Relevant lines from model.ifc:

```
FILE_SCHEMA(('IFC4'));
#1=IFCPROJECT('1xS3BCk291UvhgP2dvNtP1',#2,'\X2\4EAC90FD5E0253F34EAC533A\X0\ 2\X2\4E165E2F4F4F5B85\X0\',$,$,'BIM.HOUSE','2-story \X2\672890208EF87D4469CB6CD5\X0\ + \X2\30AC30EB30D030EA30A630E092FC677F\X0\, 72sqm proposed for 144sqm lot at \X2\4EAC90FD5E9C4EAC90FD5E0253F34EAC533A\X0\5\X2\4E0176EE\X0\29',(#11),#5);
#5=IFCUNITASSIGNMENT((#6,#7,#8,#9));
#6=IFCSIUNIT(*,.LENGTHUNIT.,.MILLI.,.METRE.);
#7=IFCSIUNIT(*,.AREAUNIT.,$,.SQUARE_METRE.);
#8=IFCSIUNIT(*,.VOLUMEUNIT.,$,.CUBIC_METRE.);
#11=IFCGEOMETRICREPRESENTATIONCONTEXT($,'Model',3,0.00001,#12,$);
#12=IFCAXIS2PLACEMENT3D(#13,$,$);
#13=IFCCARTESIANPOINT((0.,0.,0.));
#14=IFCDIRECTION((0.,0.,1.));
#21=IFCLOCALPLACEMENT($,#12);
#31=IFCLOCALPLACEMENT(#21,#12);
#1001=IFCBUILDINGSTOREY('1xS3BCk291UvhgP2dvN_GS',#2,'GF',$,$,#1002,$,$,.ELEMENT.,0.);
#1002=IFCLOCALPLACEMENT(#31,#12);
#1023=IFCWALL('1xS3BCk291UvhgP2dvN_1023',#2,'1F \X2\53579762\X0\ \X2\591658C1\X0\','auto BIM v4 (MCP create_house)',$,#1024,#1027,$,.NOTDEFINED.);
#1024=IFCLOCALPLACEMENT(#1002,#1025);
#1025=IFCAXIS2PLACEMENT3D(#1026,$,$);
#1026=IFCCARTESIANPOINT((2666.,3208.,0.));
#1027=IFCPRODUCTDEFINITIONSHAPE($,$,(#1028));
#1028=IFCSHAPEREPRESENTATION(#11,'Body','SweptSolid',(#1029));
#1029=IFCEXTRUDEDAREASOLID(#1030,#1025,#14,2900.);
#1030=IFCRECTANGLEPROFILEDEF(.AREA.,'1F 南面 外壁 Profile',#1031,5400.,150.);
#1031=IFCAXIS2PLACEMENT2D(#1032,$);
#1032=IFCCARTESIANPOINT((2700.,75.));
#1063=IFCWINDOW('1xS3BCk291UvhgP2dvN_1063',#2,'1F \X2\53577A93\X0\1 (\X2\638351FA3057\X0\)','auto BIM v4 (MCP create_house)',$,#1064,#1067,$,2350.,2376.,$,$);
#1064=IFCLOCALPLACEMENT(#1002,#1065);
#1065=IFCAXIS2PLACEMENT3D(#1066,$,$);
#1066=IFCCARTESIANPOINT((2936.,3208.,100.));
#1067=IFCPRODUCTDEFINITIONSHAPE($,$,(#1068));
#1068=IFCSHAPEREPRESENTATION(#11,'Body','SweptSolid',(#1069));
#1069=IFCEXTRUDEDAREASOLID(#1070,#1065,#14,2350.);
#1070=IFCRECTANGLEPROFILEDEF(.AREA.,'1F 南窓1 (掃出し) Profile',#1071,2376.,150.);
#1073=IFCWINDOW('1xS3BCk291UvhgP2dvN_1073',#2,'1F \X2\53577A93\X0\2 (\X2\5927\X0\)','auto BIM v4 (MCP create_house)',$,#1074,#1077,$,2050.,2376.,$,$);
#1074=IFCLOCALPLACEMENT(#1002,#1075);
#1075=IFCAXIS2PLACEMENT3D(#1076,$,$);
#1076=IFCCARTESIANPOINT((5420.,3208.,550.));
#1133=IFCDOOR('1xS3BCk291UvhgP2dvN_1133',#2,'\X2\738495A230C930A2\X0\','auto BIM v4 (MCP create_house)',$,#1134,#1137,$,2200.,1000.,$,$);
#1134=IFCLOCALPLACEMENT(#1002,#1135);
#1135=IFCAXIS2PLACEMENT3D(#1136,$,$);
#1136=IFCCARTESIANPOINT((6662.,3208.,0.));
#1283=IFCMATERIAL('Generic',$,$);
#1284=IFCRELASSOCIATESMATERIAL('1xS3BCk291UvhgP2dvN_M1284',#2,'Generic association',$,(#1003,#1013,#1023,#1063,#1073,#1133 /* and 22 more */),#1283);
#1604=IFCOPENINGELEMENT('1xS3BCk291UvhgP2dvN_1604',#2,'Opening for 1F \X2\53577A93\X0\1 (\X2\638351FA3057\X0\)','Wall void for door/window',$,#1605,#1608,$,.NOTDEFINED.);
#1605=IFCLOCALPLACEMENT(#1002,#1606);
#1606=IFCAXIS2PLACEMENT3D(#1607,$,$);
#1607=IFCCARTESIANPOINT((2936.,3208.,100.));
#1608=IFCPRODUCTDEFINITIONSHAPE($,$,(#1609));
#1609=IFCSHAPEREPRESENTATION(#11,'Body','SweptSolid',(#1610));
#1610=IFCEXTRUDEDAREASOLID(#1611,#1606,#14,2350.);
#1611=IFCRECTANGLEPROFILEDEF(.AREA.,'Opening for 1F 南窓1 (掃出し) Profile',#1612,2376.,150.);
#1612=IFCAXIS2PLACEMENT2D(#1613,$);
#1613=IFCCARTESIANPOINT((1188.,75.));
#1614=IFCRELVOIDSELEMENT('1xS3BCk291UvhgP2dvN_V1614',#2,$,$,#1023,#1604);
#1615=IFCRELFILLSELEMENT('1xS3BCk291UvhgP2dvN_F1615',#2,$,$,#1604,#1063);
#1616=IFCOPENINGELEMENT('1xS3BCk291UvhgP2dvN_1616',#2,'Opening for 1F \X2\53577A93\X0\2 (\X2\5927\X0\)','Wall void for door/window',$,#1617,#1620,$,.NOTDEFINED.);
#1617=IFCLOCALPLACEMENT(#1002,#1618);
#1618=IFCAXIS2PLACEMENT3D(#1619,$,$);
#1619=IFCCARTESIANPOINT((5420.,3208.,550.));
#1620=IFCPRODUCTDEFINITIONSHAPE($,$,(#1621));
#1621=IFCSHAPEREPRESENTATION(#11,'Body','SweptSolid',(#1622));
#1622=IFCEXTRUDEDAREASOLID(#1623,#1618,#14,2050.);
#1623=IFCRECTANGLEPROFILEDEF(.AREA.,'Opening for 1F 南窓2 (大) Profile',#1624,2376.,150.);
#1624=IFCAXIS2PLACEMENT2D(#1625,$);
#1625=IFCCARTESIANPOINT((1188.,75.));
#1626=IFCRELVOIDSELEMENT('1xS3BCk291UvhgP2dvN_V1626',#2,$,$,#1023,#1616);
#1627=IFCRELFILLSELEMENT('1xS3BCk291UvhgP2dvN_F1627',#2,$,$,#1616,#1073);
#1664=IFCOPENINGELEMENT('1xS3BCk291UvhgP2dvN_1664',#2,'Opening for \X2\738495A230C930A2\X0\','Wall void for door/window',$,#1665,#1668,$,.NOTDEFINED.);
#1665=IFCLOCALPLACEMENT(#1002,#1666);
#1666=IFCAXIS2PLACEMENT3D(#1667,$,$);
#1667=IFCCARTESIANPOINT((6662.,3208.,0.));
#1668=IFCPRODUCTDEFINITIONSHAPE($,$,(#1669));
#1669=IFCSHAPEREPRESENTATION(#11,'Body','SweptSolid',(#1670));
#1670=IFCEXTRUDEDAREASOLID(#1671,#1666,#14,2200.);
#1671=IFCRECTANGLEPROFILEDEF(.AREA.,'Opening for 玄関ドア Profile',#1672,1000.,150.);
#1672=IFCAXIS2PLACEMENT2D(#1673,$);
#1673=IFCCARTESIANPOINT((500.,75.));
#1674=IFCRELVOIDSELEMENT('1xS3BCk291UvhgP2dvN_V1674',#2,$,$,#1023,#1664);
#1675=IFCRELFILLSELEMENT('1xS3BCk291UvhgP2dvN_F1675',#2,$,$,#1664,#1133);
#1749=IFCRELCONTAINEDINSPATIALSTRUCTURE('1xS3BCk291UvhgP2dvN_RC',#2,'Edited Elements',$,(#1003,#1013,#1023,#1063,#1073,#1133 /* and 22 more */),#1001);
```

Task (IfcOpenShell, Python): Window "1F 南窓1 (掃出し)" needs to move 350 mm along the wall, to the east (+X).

```python
import ifcopenshell
import ifcopenshell.api.geometry
import ifcopenshell.util.placement
import ifcopenshell.util.unit

model = ifcopenshell.open("model.ifc")
unit_scale = ifcopenshell.util.unit.calculate_unit_scale(model)

window = model.by_guid("1xS3BCk291UvhgP2dvN_1063")
opening = window.FillsVoids[0].RelatingOpeningElement
wall = opening.VoidsElements[0].RelatingBuildingElement

wall_matrix = ifcopenshell.util.placement.get_local_placement(wall.ObjectPlacement)
shift = wall_matrix[:3, 0] * 0.35 / unit_scale
before = ifcopenshell.util.placement.get_local_placement(window.ObjectPlacement)[:3, 3].copy()

# The window is not placed relative to its opening, so move both.
for product in (opening, window):
    matrix = ifcopenshell.util.placement.get_local_placement(product.ObjectPlacement)
    matrix[:3, 3] += shift
    ifcopenshell.api.geometry.edit_object_placement(model, product=product, matrix=matrix, is_si=False)

after = ifcopenshell.util.placement.get_local_placement(window.ObjectPlacement)[:3, 3]
print("window moved by", (after - before).round(3) + 0.0)

model.write("model-out.ifc")
```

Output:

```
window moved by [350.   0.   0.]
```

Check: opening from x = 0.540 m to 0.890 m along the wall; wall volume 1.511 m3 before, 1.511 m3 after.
